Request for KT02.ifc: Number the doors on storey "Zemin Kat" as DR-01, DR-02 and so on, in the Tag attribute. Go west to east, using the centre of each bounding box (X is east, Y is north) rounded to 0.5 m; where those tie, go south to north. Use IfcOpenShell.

First a look at what the model holds.

```python
import ifcopenshell
import ifcopenshell.util.element
import ifcopenshell.util.placement

model = ifcopenshell.open("KT02.ifc")
print(model.schema)
storey = next(s for s in model.by_type("IfcBuildingStorey") if s.Name == "Zemin Kat")
doors = [e for e in ifcopenshell.util.element.get_decomposition(storey) if e.is_a("IfcDoor")]
for e in sorted(doors, key=lambda e: e.id()):
    origin = ifcopenshell.util.placement.get_local_placement(e.ObjectPlacement)[:3, 3]
    print(e.id(), e.Tag, e.Name, origin.round(2) + 0.0, sep=" | ")
```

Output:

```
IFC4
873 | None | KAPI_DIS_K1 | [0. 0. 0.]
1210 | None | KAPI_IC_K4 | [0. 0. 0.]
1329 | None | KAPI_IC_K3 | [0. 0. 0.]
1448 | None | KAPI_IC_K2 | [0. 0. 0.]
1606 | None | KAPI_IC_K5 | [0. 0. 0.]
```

```python
import ifcopenshell
import ifcopenshell.geom
import ifcopenshell.util.element
import ifcopenshell.util.shape

model = ifcopenshell.open("KT02.ifc")
settings = ifcopenshell.geom.settings()
settings.set("use-world-coords", True)


def centre(element):
    shape = ifcopenshell.geom.create_shape(settings, element)
    return ifcopenshell.util.shape.get_bbox_centroid(shape.geometry)


storey = next(s for s in model.by_type("IfcBuildingStorey") if s.Name == "Zemin Kat")
doors = [e for e in ifcopenshell.util.element.get_decomposition(storey) if e.is_a("IfcDoor")]

# Insertion points can sit at a corner or the storey origin, so sort by the geometry (in metres).
centres = {e: centre(e) for e in doors}
doors.sort(key=lambda e: (round(centres[e][0] / 0.5), centres[e][1]))

for i, e in enumerate(doors, start=1):
    number = f"DR-{i:02d}"
    e.Tag = number
    print(e.id(), number)

model.write("KT02_v2.ifc")
```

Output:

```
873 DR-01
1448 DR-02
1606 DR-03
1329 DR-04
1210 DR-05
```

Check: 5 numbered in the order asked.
